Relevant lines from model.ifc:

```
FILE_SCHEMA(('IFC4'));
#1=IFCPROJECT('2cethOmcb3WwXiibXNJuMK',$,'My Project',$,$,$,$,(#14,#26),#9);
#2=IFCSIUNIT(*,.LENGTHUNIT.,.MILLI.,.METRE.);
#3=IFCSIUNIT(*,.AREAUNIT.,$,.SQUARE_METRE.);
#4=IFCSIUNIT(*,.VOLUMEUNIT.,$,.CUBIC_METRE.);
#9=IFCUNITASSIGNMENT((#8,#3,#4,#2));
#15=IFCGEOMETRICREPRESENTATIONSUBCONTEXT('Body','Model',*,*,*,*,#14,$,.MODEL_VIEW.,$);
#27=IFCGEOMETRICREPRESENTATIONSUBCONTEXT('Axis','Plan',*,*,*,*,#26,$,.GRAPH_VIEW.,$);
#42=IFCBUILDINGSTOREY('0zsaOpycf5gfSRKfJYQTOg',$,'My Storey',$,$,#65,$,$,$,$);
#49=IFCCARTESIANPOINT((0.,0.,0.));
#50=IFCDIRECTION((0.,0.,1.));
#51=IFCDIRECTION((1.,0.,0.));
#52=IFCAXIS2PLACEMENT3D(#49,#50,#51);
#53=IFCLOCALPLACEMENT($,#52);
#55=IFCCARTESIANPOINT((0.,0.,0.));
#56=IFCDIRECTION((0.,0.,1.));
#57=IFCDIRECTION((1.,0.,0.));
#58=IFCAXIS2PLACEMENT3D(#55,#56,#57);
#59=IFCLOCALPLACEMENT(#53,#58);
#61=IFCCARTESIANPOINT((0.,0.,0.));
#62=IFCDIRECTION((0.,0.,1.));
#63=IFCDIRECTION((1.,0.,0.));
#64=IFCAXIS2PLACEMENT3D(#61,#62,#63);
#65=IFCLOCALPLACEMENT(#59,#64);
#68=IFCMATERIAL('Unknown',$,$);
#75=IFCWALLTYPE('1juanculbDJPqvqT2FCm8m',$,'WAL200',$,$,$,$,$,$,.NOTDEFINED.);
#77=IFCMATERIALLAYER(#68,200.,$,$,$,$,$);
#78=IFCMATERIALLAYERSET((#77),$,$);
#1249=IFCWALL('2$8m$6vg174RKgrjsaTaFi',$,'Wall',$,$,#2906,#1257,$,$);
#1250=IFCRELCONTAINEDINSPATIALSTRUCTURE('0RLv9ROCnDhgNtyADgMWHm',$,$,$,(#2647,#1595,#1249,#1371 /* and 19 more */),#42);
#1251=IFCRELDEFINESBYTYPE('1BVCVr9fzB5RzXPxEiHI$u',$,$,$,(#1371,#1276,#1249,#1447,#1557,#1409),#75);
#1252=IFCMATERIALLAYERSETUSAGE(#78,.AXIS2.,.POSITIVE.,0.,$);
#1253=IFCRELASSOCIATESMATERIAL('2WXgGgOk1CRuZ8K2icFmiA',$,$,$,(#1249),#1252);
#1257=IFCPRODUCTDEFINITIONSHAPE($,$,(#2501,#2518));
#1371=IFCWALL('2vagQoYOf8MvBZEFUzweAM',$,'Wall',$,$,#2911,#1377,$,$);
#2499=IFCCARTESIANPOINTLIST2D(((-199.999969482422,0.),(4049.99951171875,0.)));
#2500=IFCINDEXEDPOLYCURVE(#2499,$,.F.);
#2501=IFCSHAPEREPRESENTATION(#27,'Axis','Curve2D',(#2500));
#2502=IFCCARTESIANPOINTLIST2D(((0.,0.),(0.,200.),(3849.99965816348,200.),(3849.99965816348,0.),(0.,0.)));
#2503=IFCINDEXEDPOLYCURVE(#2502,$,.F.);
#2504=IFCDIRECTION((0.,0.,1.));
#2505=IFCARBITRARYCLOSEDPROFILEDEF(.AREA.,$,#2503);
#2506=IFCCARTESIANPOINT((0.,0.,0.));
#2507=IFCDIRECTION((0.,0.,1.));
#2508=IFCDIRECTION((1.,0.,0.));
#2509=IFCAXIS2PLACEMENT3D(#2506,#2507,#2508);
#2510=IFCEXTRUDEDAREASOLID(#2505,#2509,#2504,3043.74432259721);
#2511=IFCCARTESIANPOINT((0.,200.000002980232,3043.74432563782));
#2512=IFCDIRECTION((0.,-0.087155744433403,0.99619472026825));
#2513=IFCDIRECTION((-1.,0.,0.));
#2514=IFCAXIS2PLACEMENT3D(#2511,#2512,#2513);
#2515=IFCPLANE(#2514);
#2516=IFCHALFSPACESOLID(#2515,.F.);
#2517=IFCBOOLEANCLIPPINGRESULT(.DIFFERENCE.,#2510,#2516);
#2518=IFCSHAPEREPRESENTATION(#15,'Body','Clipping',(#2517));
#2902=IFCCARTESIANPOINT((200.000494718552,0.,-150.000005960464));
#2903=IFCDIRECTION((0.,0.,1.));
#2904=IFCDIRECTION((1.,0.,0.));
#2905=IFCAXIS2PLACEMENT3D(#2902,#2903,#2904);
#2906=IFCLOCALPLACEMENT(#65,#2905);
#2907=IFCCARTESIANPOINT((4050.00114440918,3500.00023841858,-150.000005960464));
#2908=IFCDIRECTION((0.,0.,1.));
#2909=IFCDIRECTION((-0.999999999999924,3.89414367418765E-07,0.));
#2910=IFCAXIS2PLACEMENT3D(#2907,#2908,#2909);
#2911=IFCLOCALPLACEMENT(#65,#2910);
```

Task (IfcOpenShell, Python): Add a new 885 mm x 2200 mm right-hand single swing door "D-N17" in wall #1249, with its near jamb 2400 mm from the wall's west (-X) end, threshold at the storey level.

```python
import numpy as np
import ifcopenshell
import ifcopenshell.api.feature
import ifcopenshell.api.geometry
import ifcopenshell.api.root
import ifcopenshell.api.spatial
import ifcopenshell.geom
import ifcopenshell.util.element
import ifcopenshell.util.placement
import ifcopenshell.util.representation
import ifcopenshell.util.shape
import ifcopenshell.util.unit

model = ifcopenshell.open("model.ifc")
unit_scale = ifcopenshell.util.unit.calculate_unit_scale(model)
settings = ifcopenshell.geom.settings()


def volume(element):
    """Net volume in cubic metres, openings subtracted."""
    shape = ifcopenshell.geom.create_shape(settings, element)
    return ifcopenshell.util.shape.get_volume(shape.geometry)


wall = model.by_guid("2$8m$6vg174RKgrjsaTaFi")
storey = ifcopenshell.util.element.get_container(wall, ifc_class="IfcBuildingStorey")
context = ifcopenshell.util.representation.get_context(model, "Model", "Body", "MODEL_VIEW")
before = volume(wall)

width, height, from_end, sill = 0.885, 2.2, 2.4, 0.0  # metres

# The wall runs along its own X axis, and the end named is its -X end.
wall_shape = ifcopenshell.geom.create_shape(settings, wall)
x, y, z = ifcopenshell.util.shape.get_vertices(wall_shape.geometry).T
start = x.min() + from_end
face, thickness = float(y.min()), float(y.max() - y.min())
wall_matrix = ifcopenshell.util.placement.get_local_placement(wall.ObjectPlacement)
level = ifcopenshell.util.placement.get_local_placement(storey.ObjectPlacement)[2, 3]


def in_wall(x, y):
    """Placement at x, y metres in the wall's axes, at sill height."""
    matrix = wall_matrix.copy()
    matrix[:, 3] = wall_matrix @ np.array([x / unit_scale, y / unit_scale, 0.0, 1.0])
    matrix[2, 3] = level + sill / unit_scale
    return matrix


# Opening: a box that overshoots both wall faces by 50 mm.
opening = ifcopenshell.api.root.create_entity(model, ifc_class="IfcOpeningElement", predefined_type="OPENING")
box = ifcopenshell.api.geometry.add_wall_representation(
    model, context=context, length=width, height=height, thickness=thickness + 0.1
)
ifcopenshell.api.geometry.assign_representation(model, product=opening, representation=box)
ifcopenshell.api.geometry.edit_object_placement(model, product=opening, matrix=in_wall(start, face - 0.05), is_si=False)
ifcopenshell.api.feature.add_feature(model, feature=opening, element=wall)

door = ifcopenshell.api.root.create_entity(model, ifc_class="IfcDoor", name="D-N17", predefined_type="DOOR")
door.OverallWidth, door.OverallHeight = width / unit_scale, height / unit_scale
door.OperationType = "SINGLE_SWING_RIGHT"
body = ifcopenshell.api.geometry.add_door_representation(
    model,
    context=context,
    overall_width=door.OverallWidth,
    overall_height=door.OverallHeight,
    operation_type="SINGLE_SWING_RIGHT",
    lining_properties={"LiningDepth": thickness / unit_scale, "ThresholdDepth": thickness / unit_scale},
)
ifcopenshell.api.geometry.assign_representation(model, product=door, representation=body)
ifcopenshell.api.spatial.assign_container(model, products=[door], relating_structure=storey)
ifcopenshell.api.feature.add_filling(model, opening=opening, element=door)

# The lining spans the wall, so the door starts at the wall face.
ifcopenshell.api.geometry.edit_object_placement(model, product=door, matrix=in_wall(start, face), is_si=False)

after = volume(wall)

print(f"wall volume {before:.3f} -> {after:.3f} m3")

model.write("model-out.ifc")
```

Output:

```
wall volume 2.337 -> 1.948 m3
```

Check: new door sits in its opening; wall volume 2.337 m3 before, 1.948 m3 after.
